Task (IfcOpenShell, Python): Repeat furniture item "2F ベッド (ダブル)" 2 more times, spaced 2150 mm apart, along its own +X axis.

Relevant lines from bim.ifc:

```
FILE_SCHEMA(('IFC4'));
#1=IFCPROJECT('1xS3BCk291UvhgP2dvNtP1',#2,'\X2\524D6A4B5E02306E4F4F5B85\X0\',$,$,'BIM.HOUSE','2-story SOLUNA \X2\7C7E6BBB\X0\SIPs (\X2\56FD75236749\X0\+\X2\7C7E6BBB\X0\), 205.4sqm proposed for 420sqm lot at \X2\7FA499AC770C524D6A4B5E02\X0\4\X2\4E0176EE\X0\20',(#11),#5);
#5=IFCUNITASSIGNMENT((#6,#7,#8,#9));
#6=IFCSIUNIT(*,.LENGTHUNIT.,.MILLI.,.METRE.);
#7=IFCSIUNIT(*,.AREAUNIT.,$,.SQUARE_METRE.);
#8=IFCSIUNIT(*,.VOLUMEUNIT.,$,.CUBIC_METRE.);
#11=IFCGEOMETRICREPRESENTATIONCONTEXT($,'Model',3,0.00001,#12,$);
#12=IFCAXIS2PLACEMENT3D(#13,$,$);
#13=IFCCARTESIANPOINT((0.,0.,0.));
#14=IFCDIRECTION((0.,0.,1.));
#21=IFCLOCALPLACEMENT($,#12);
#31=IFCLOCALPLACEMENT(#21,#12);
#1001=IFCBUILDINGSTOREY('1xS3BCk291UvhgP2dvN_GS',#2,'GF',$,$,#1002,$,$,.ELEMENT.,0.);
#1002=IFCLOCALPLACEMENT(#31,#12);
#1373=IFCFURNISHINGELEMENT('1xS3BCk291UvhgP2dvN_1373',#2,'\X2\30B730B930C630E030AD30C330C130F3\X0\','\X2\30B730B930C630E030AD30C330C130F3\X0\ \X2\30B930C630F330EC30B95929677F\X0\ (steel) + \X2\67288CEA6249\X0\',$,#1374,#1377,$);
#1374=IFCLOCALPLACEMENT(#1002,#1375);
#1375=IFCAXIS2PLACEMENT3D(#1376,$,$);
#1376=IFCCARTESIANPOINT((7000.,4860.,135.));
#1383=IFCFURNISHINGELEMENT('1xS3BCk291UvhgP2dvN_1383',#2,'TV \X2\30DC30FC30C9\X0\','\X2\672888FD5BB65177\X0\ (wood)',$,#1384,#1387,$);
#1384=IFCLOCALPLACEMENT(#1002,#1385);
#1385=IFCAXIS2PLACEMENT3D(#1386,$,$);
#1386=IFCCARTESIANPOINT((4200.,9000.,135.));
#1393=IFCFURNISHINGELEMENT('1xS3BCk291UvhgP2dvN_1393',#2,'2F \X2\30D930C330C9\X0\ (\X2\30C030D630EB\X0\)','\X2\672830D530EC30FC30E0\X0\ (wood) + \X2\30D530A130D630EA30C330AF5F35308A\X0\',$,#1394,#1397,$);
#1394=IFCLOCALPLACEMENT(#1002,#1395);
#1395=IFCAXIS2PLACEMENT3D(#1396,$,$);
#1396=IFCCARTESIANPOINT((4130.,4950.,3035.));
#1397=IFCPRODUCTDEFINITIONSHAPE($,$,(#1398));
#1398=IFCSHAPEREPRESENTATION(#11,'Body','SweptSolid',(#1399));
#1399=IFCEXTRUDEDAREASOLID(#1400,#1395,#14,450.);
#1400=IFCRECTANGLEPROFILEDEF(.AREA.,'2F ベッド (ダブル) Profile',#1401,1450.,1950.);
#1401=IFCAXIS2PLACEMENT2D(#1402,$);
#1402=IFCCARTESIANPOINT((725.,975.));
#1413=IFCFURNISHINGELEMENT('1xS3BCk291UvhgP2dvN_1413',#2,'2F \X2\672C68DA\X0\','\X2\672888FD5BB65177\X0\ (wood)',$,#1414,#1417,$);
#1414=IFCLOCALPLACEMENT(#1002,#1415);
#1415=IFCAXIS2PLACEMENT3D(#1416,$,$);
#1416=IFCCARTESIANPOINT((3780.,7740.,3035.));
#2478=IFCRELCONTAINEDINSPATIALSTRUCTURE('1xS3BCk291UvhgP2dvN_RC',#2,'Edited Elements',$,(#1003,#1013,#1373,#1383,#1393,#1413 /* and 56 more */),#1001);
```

```python
import ifcopenshell
import ifcopenshell.api.geometry
import ifcopenshell.api.root
import ifcopenshell.util.element
import ifcopenshell.util.placement

model = ifcopenshell.open("bim.ifc")


def reuse_history(source, copy):
    """copy_class also copies each property set's owner history, people and application; keep the originals."""
    for rel in copy.IsDefinedBy:
        if rel.is_a("IfcRelDefinesByProperties") and (history := rel.RelatingPropertyDefinition.OwnerHistory):
            rel.RelatingPropertyDefinition.OwnerHistory = source.OwnerHistory
            ifcopenshell.util.element.remove_deep2(model, history)


source = model.by_id(1393)
base = ifcopenshell.util.placement.get_local_placement(source.ObjectPlacement)
step = base[:3, 0] * 2150.0

for i in range(1, 3):
    copy = ifcopenshell.api.root.copy_class(model, product=source)
    copy.Representation = ifcopenshell.util.element.copy_deep(
        model, source.Representation, exclude=["IfcGeometricRepresentationContext", "IfcRepresentationMap"]
    )
    reuse_history(source, copy)
    matrix = base.copy()
    matrix[:3, 3] += i * step
    print("added at", matrix[:3, 3].round(3) + 0.0)
    ifcopenshell.api.geometry.edit_object_placement(model, product=copy, matrix=matrix, is_si=False)

model.write("bim_updated.ifc")
```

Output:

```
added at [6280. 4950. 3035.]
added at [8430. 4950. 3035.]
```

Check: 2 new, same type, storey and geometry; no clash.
